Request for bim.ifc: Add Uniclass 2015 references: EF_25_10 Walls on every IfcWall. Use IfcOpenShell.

First a look at what the model holds.

```python
import ifcopenshell

model = ifcopenshell.open("bim.ifc")
print(model.schema)
print("classifications:", [c.Name for c in model.by_type("IfcClassification")])
for ifc_class in ("IfcDoor", "IfcRoof", "IfcStair", "IfcWall", "IfcWindow"):
    print(ifc_class, len(model.by_type(ifc_class)))
```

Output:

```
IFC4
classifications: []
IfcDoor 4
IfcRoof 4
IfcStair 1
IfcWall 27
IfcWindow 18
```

```python
import ifcopenshell
import ifcopenshell.api.classification

model = ifcopenshell.open("bim.ifc")

system = ifcopenshell.api.classification.add_classification(model, classification="Uniclass 2015")

codes = {
    "IfcWall": ("EF_25_10", "Walls"),
}
for ifc_class, (code, name) in codes.items():
    products = model.by_type(ifc_class)
    ifcopenshell.api.classification.add_reference(
        model, products=products, classification=system, identification=code, name=name
    )
    print(code, len(products))

model.write("bim-out.ifc")
```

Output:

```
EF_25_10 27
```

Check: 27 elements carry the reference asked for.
